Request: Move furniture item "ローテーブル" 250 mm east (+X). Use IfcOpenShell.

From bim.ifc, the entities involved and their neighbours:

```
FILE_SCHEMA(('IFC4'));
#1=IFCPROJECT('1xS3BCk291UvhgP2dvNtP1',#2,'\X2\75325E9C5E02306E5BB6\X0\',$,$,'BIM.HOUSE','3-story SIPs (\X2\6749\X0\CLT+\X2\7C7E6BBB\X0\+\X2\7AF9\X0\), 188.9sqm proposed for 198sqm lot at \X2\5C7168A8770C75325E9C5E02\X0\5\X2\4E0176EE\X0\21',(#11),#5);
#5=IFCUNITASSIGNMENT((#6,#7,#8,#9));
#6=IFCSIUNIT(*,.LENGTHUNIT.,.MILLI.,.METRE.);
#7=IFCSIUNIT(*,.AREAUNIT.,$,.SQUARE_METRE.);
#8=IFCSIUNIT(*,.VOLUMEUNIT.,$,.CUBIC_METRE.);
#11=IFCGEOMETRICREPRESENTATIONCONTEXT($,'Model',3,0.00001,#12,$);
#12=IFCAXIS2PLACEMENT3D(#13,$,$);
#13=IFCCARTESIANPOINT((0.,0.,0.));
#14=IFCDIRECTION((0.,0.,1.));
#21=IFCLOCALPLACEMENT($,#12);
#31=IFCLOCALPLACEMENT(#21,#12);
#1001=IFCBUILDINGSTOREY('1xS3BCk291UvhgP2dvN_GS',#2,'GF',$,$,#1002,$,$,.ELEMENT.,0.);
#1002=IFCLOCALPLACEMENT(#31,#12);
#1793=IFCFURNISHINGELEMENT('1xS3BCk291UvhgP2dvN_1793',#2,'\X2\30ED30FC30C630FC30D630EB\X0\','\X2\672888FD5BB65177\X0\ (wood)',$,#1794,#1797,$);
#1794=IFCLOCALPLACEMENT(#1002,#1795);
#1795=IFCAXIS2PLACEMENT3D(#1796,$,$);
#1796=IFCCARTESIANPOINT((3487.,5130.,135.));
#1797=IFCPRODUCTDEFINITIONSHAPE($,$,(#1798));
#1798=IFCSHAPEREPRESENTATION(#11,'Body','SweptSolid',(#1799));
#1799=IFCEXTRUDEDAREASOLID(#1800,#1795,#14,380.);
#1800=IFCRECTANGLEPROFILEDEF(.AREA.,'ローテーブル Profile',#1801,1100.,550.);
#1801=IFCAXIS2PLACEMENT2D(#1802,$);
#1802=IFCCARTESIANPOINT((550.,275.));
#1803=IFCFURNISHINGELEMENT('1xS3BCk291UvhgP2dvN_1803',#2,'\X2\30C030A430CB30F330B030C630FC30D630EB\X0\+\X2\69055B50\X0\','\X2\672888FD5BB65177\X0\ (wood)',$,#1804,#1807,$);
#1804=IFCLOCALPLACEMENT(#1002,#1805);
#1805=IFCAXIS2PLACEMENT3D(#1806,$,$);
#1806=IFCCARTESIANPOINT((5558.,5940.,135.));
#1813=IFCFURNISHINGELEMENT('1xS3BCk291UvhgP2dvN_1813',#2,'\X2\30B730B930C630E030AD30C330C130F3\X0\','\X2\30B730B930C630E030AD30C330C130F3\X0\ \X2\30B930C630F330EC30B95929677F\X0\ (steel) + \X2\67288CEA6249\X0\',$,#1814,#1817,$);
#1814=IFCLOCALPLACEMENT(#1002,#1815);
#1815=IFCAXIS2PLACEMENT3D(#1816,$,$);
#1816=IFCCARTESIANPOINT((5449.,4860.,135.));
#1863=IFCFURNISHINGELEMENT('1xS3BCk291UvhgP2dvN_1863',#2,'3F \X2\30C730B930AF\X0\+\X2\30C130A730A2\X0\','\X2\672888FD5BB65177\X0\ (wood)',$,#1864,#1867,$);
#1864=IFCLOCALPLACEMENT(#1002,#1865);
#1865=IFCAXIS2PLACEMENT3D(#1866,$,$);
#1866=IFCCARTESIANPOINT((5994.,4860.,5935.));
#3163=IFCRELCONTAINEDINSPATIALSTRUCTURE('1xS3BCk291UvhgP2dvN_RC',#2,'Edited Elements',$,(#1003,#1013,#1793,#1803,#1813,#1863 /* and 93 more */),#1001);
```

```python
import ifcopenshell
import ifcopenshell.api.geometry
import ifcopenshell.util.placement

model = ifcopenshell.open("bim.ifc")

item = model.by_guid("1xS3BCk291UvhgP2dvN_1793")
matrix = ifcopenshell.util.placement.get_local_placement(item.ObjectPlacement)
matrix[0, 3] += 250.0
ifcopenshell.api.geometry.edit_object_placement(model, product=item, matrix=matrix, is_si=False)

print(ifcopenshell.util.placement.get_local_placement(item.ObjectPlacement).round(3) + 0.0)

model.write("bim_edited.ifc")
```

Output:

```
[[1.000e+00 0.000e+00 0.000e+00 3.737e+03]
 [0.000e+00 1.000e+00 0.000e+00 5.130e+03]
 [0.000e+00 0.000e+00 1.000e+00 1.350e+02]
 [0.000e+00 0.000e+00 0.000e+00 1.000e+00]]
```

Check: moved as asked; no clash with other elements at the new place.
